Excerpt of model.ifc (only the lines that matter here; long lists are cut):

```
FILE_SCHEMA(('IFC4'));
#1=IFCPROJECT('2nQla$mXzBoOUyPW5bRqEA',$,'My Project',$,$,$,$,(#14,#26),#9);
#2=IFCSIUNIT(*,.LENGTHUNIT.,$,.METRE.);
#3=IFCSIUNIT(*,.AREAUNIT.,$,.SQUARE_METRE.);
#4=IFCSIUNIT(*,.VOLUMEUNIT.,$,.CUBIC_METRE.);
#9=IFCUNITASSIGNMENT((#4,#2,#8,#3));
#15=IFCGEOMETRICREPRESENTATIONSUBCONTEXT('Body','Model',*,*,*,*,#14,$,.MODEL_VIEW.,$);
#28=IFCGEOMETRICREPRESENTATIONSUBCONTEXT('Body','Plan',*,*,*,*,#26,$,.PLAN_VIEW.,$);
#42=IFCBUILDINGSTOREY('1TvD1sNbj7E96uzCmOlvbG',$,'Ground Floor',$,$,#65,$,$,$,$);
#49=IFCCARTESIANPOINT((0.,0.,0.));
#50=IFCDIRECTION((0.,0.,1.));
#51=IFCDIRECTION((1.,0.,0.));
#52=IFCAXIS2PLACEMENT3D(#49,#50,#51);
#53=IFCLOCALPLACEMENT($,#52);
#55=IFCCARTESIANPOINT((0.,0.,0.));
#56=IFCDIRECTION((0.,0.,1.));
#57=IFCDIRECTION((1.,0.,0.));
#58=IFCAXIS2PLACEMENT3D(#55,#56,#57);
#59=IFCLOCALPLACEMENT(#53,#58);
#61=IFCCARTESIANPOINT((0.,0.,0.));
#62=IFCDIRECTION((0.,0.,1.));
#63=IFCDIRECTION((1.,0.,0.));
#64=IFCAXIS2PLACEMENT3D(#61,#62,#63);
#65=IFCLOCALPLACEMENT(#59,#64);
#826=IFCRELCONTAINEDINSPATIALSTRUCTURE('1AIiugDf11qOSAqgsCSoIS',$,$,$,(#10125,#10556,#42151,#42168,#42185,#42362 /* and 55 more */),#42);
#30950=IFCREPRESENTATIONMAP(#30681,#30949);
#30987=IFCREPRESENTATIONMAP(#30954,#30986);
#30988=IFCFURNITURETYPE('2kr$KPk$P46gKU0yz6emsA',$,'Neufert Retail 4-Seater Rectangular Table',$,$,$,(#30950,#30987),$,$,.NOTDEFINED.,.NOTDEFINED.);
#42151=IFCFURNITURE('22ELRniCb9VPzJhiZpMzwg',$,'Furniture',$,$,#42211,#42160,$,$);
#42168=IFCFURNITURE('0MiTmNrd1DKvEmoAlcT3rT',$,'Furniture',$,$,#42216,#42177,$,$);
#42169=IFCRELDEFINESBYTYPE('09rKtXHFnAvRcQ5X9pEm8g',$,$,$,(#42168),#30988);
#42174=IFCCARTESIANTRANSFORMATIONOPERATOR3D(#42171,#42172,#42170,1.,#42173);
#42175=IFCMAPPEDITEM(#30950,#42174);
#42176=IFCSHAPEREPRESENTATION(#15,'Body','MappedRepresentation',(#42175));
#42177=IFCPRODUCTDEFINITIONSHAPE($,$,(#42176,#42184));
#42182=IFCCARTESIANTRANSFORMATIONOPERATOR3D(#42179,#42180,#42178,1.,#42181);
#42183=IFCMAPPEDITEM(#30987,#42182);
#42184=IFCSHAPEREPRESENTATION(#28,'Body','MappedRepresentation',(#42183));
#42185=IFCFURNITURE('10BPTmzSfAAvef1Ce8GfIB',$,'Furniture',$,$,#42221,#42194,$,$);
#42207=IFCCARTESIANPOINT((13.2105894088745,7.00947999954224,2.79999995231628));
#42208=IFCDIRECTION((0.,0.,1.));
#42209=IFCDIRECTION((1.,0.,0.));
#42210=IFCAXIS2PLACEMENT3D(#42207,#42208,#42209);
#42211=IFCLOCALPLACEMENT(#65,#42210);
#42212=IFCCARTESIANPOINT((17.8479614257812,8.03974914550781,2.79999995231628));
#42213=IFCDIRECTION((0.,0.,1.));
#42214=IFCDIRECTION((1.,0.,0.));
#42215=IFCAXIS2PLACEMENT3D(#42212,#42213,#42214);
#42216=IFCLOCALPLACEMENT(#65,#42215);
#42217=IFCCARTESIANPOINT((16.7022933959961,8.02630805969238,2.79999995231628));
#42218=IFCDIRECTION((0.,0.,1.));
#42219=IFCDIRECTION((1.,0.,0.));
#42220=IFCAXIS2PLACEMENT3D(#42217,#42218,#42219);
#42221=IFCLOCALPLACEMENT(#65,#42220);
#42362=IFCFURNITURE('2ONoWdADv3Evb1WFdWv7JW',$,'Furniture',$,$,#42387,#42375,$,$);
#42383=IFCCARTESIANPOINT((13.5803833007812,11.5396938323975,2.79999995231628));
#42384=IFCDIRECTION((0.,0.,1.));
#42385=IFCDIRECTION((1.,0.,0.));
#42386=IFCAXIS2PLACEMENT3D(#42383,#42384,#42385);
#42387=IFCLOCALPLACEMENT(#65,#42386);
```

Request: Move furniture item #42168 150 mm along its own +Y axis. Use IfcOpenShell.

```python
import ifcopenshell
import ifcopenshell.api.geometry
import ifcopenshell.util.placement
import ifcopenshell.util.unit

model = ifcopenshell.open("model.ifc")
unit_scale = ifcopenshell.util.unit.calculate_unit_scale(model)

item = model.by_guid("0MiTmNrd1DKvEmoAlcT3rT")
matrix = ifcopenshell.util.placement.get_local_placement(item.ObjectPlacement)
matrix[:3, 3] += matrix[:3, 1] * 0.15 / unit_scale
ifcopenshell.api.geometry.edit_object_placement(model, product=item, matrix=matrix, is_si=False)

print(ifcopenshell.util.placement.get_local_placement(item.ObjectPlacement).round(3) + 0.0)

model.write("model-out.ifc")
```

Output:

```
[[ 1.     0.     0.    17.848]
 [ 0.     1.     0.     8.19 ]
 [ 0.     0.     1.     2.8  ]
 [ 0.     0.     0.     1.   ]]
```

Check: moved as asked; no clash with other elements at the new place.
